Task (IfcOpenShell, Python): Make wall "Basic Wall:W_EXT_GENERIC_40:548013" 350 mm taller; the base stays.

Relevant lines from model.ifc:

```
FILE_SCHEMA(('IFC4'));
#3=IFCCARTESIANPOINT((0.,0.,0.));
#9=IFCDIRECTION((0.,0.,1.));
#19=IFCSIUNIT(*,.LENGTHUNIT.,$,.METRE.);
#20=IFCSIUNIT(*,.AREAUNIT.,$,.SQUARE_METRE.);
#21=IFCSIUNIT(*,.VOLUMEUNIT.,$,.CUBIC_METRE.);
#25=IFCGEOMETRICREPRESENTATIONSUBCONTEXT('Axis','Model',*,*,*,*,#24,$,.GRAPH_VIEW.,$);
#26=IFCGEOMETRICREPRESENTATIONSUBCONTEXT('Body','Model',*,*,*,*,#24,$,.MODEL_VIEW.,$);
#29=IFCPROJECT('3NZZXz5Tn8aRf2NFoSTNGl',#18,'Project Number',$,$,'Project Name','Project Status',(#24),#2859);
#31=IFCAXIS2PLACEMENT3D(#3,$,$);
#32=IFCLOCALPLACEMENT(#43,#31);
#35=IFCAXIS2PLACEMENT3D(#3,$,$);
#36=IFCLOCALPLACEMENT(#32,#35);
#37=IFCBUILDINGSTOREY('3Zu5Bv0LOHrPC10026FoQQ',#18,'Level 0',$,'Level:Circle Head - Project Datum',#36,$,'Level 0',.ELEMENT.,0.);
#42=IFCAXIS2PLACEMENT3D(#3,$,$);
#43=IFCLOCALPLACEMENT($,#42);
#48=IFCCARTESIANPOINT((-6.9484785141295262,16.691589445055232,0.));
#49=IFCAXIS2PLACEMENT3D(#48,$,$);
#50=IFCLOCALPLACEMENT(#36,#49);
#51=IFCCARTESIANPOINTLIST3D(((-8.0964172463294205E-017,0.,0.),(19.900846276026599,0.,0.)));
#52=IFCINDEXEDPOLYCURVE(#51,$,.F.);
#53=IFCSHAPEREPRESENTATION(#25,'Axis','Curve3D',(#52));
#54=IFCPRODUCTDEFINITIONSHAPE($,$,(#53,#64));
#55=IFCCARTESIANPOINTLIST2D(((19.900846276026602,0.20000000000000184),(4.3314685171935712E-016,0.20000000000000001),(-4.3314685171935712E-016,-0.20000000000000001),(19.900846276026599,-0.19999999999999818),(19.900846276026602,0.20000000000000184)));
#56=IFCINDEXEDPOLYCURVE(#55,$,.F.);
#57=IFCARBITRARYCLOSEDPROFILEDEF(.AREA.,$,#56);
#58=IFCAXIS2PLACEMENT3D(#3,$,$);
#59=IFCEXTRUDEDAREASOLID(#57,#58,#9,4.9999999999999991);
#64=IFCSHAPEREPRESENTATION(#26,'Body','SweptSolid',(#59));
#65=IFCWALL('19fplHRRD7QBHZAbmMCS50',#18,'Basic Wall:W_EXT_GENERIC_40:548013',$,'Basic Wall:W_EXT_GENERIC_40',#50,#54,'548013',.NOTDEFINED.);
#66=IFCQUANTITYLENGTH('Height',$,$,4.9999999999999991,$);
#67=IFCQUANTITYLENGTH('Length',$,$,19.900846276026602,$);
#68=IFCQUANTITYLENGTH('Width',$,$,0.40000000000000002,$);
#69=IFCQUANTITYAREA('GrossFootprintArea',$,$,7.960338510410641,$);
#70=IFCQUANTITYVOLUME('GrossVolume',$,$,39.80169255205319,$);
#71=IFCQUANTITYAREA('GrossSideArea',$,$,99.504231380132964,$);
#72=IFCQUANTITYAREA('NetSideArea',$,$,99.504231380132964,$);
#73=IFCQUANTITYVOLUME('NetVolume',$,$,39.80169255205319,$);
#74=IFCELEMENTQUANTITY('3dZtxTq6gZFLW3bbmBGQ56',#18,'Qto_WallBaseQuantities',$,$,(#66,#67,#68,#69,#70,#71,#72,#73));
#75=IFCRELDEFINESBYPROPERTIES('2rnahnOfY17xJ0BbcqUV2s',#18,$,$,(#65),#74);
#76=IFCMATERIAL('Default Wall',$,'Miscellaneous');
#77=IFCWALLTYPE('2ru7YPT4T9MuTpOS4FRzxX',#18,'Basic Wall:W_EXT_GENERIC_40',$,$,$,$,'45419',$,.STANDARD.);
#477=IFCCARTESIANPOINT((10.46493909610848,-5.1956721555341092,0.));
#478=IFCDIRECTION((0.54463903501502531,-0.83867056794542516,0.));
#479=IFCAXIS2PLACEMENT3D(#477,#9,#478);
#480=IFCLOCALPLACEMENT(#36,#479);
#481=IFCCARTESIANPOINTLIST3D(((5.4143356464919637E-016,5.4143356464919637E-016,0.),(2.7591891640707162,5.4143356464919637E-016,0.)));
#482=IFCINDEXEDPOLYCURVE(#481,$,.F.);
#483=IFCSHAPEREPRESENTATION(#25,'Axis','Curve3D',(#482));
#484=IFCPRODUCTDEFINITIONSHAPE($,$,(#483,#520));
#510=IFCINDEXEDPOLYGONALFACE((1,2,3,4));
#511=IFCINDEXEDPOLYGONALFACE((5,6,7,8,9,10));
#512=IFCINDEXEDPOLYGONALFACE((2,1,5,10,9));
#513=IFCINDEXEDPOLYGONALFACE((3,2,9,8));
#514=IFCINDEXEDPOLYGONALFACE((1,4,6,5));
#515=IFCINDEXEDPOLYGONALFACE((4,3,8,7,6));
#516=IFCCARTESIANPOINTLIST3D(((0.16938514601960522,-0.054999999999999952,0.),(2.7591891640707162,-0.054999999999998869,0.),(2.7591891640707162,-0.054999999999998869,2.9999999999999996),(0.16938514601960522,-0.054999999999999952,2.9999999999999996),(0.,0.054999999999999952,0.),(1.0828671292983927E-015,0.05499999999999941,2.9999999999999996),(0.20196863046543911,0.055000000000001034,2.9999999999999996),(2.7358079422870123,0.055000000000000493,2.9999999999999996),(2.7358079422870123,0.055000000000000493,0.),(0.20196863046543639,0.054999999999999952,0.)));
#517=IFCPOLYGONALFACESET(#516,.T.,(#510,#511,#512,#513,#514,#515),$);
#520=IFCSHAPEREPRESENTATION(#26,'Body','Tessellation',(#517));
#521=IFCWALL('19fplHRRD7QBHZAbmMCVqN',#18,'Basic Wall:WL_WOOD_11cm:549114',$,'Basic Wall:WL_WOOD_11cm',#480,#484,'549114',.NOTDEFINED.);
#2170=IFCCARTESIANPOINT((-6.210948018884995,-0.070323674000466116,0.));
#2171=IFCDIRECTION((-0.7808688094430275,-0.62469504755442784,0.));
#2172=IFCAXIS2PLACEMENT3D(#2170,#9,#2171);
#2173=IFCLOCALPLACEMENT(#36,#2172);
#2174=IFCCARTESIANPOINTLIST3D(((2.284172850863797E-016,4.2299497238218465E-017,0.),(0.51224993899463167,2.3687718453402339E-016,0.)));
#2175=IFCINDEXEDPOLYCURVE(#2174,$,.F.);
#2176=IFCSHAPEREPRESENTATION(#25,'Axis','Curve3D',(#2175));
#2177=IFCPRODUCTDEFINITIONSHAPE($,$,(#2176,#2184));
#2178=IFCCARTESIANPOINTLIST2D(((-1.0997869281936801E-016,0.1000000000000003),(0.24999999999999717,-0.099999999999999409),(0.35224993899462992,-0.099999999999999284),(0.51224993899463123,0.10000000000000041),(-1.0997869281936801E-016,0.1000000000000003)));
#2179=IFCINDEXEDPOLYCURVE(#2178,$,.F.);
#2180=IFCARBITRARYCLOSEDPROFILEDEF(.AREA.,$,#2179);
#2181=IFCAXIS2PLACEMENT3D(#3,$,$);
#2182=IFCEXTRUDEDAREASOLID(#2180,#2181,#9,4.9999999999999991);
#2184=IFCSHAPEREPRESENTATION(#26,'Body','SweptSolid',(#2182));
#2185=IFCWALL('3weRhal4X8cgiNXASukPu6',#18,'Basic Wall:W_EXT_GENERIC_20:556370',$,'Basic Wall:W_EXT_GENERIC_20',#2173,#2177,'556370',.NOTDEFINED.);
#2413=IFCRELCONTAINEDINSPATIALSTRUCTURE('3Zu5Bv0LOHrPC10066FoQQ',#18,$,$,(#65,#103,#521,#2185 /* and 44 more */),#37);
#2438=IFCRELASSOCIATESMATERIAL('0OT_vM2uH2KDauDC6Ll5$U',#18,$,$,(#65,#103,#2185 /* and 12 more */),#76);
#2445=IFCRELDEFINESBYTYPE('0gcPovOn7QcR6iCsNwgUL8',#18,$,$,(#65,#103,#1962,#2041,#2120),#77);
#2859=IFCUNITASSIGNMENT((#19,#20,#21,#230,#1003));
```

```python
import ifcopenshell
import ifcopenshell.api.pset
import ifcopenshell.geom
import ifcopenshell.util.element
import ifcopenshell.util.representation
import ifcopenshell.util.shape
import ifcopenshell.util.unit

model = ifcopenshell.open("model.ifc")
unit_scale = ifcopenshell.util.unit.calculate_unit_scale(model)
area_scale = ifcopenshell.util.unit.calculate_unit_scale(model, "AREAUNIT")
volume_scale = ifcopenshell.util.unit.calculate_unit_scale(model, "VOLUMEUNIT")
settings = ifcopenshell.geom.settings()


def volume(element):
    """Net volume in cubic metres, openings subtracted."""
    shape = ifcopenshell.geom.create_shape(settings, element)
    return ifcopenshell.util.shape.get_volume(shape.geometry)


wall = model.by_id(65)
before = volume(wall)

body = ifcopenshell.util.representation.get_representation(wall, "Model", "Body")
solid = body.Items[0]
old_height = solid.Depth
solid.Depth += 0.35 / unit_scale
after = volume(wall)
thickness = 0.4  # wall thickness in metres

# Update the stored height, areas and volumes.
qto = model.by_id(ifcopenshell.util.element.get_pset(wall, "Qto_WallBaseQuantities", should_inherit=False)["id"])
ifcopenshell.api.pset.edit_qto(model, qto=qto, properties={
    "Height": solid.Depth,
    "GrossVolume": ifcopenshell.util.element.get_pset(wall, "Qto_WallBaseQuantities", "GrossVolume") * solid.Depth / old_height,
    "GrossSideArea": ifcopenshell.util.element.get_pset(wall, "Qto_WallBaseQuantities", "GrossSideArea") * solid.Depth / old_height,
    "NetSideArea": after / thickness / area_scale,
    "NetVolume": after / volume_scale,
})

print(f"height {old_height:g} -> {solid.Depth:g}, volume {before:.3f} -> {after:.3f} m3")

model.write("model_updated.ifc")
```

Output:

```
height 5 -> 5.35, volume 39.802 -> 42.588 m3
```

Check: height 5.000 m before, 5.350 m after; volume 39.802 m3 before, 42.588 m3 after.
